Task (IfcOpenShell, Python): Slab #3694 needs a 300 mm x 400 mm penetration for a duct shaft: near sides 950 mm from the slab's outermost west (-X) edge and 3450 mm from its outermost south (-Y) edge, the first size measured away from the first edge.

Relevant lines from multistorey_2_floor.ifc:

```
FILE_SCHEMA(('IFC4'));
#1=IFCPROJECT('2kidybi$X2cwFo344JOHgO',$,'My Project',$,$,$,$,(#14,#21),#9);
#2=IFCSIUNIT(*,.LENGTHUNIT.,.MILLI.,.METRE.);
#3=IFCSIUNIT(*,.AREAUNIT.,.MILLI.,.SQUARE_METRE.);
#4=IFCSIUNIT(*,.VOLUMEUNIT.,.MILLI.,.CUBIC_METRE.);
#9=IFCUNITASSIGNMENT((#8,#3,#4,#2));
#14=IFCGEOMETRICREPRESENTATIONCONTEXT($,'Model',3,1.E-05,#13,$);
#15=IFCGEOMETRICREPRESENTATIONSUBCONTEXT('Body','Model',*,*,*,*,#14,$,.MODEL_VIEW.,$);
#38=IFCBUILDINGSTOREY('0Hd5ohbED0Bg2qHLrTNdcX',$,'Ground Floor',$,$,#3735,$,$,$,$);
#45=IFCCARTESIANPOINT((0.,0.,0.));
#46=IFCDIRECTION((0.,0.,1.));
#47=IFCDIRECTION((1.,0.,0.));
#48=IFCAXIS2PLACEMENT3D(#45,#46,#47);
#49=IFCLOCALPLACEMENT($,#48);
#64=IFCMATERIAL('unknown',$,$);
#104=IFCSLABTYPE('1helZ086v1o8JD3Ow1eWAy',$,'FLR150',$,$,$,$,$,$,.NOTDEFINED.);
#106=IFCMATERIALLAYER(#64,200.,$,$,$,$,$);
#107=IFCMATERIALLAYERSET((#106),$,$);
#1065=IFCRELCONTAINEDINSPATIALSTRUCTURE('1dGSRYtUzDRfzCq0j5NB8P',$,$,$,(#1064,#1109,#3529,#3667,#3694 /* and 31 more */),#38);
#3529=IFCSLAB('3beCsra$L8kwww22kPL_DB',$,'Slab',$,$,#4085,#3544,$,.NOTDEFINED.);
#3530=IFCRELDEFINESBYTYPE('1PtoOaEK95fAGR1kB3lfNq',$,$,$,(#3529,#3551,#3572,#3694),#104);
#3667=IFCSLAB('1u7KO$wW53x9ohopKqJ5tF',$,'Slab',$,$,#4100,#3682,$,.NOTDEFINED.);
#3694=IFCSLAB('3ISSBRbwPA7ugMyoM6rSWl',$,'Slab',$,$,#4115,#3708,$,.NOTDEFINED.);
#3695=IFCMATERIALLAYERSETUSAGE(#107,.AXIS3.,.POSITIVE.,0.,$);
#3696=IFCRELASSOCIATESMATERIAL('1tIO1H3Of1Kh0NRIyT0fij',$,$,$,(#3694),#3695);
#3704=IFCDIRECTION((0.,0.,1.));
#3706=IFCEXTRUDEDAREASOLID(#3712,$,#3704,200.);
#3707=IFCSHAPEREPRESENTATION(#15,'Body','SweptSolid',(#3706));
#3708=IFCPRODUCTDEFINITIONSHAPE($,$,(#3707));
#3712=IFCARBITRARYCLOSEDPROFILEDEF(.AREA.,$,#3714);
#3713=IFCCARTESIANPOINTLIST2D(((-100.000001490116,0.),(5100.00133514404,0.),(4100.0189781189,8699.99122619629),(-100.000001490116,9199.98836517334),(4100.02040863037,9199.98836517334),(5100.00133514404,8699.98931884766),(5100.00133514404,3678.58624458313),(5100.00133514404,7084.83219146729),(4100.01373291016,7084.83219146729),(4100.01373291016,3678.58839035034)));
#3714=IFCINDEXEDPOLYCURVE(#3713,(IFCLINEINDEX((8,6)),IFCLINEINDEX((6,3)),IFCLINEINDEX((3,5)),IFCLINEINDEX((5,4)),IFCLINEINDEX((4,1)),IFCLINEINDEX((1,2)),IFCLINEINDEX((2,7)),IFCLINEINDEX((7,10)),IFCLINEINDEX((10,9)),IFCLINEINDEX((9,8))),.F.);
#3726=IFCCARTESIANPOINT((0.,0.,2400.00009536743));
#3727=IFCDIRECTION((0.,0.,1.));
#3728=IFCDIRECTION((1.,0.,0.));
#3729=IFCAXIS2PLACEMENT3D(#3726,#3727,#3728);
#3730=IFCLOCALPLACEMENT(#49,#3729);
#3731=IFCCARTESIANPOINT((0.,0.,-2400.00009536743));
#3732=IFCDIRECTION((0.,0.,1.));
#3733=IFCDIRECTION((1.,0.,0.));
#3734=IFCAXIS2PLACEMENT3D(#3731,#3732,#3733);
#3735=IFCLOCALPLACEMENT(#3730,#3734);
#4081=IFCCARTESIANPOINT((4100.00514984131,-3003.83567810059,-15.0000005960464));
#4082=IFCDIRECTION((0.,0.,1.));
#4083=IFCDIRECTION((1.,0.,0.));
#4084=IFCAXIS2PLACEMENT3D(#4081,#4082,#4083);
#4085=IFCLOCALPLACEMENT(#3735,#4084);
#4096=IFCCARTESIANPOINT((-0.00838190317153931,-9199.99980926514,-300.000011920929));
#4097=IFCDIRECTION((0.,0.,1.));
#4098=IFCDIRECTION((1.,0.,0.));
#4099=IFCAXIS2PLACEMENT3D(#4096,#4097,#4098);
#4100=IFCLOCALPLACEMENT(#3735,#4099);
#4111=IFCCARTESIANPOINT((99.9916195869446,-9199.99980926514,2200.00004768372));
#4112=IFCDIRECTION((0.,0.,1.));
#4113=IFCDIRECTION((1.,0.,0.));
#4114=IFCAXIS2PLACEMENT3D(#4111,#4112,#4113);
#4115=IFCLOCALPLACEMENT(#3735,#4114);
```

```python
import numpy as np
import ifcopenshell
import ifcopenshell.api.feature
import ifcopenshell.api.geometry
import ifcopenshell.api.root
import ifcopenshell.geom
import ifcopenshell.util.placement
import ifcopenshell.util.representation
import ifcopenshell.util.shape
import ifcopenshell.util.unit

model = ifcopenshell.open("multistorey_2_floor.ifc")
unit_scale = ifcopenshell.util.unit.calculate_unit_scale(model)
settings = ifcopenshell.geom.settings()


def volume(element):
    """Net volume in cubic metres, openings subtracted."""
    shape = ifcopenshell.geom.create_shape(settings, element)
    return ifcopenshell.util.shape.get_volume(shape.geometry)


slab = model.by_guid("3ISSBRbwPA7ugMyoM6rSWl")
before = volume(slab)

# Extent in the slab's own axes, in metres. The edges named are its -X and -Y sides.
slab_shape = ifcopenshell.geom.create_shape(settings, slab)
vertices = ifcopenshell.util.shape.get_vertices(slab_shape.geometry)
x_min, y_min, bottom = vertices.min(axis=0)
top = vertices[:, 2].max()

opening = ifcopenshell.api.root.create_entity(model, ifc_class="IfcOpeningElement", name="Duct shaft opening", predefined_type="OPENING")
context = ifcopenshell.util.representation.get_context(model, "Model", "Body", "MODEL_VIEW")
width, depth = 0.3, 0.4
outline = [(0.0, 0.0), (width, 0.0), (width, depth), (0.0, depth), (0.0, 0.0)]
# Overshoot both faces by 50 mm so the cut is clean.
shape = ifcopenshell.api.geometry.add_slab_representation(
    model, context=context, depth=top - bottom + 0.1, polyline=outline
)
ifcopenshell.api.geometry.assign_representation(model, product=opening, representation=shape)

matrix = ifcopenshell.util.placement.get_local_placement(slab.ObjectPlacement)
matrix[:, 3] = matrix @ np.append(np.array([x_min + 0.95, y_min + 3.45, bottom - 0.05]) / unit_scale, 1.0)
ifcopenshell.api.geometry.edit_object_placement(model, product=opening, matrix=matrix, is_si=False)
ifcopenshell.api.feature.add_feature(model, feature=opening, element=slab)

after = volume(slab)

print(f"slab volume {before:.3f} -> {after:.3f} m3")

model.write("multistorey_2_floor-out.ifc")
```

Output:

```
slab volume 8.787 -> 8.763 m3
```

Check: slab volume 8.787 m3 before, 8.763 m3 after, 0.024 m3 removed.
